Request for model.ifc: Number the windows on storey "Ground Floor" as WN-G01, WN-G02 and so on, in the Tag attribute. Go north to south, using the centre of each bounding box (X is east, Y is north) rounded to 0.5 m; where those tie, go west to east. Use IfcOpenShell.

First a look at what the model holds.

```python
import ifcopenshell
import ifcopenshell.util.element
import ifcopenshell.util.placement

model = ifcopenshell.open("model.ifc")
print(model.schema)
storey = next(s for s in model.by_type("IfcBuildingStorey") if s.Name == "Ground Floor")
windows = [e for e in ifcopenshell.util.element.get_decomposition(storey) if e.is_a("IfcWindow")]
for e in sorted(windows, key=lambda e: e.id()):
    origin = ifcopenshell.util.placement.get_local_placement(e.ObjectPlacement)[:3, 3]
    print(e.id(), e.Tag, e.Name, origin.round(2) + 0.0, sep=" | ")
```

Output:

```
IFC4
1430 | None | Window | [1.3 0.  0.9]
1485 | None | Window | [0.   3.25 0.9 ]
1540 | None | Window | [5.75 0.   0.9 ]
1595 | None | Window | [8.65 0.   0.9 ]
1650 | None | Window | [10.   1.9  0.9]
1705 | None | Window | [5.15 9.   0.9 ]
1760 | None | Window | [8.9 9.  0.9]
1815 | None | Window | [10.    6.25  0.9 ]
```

```python
import ifcopenshell
import ifcopenshell.geom
import ifcopenshell.util.element
import ifcopenshell.util.shape

model = ifcopenshell.open("model.ifc")
settings = ifcopenshell.geom.settings()
settings.set("use-world-coords", True)


def centre(element):
    shape = ifcopenshell.geom.create_shape(settings, element)
    return ifcopenshell.util.shape.get_bbox_centroid(shape.geometry)


storey = next(s for s in model.by_type("IfcBuildingStorey") if s.Name == "Ground Floor")
windows = [e for e in ifcopenshell.util.element.get_decomposition(storey) if e.is_a("IfcWindow")]

# Insertion points can sit at a corner or the storey origin, so sort by the geometry (in metres).
centres = {e: centre(e) for e in windows}
windows.sort(key=lambda e: (-round(centres[e][1] / 0.5), centres[e][0]))

for i, e in enumerate(windows, start=1):
    number = f"WN-G{i:02d}"
    e.Tag = number
    print(e.id(), number)

model.write("model_edited.ifc")
```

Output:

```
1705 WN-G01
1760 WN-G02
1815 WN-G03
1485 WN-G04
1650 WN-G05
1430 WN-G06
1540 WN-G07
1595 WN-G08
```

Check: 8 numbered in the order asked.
